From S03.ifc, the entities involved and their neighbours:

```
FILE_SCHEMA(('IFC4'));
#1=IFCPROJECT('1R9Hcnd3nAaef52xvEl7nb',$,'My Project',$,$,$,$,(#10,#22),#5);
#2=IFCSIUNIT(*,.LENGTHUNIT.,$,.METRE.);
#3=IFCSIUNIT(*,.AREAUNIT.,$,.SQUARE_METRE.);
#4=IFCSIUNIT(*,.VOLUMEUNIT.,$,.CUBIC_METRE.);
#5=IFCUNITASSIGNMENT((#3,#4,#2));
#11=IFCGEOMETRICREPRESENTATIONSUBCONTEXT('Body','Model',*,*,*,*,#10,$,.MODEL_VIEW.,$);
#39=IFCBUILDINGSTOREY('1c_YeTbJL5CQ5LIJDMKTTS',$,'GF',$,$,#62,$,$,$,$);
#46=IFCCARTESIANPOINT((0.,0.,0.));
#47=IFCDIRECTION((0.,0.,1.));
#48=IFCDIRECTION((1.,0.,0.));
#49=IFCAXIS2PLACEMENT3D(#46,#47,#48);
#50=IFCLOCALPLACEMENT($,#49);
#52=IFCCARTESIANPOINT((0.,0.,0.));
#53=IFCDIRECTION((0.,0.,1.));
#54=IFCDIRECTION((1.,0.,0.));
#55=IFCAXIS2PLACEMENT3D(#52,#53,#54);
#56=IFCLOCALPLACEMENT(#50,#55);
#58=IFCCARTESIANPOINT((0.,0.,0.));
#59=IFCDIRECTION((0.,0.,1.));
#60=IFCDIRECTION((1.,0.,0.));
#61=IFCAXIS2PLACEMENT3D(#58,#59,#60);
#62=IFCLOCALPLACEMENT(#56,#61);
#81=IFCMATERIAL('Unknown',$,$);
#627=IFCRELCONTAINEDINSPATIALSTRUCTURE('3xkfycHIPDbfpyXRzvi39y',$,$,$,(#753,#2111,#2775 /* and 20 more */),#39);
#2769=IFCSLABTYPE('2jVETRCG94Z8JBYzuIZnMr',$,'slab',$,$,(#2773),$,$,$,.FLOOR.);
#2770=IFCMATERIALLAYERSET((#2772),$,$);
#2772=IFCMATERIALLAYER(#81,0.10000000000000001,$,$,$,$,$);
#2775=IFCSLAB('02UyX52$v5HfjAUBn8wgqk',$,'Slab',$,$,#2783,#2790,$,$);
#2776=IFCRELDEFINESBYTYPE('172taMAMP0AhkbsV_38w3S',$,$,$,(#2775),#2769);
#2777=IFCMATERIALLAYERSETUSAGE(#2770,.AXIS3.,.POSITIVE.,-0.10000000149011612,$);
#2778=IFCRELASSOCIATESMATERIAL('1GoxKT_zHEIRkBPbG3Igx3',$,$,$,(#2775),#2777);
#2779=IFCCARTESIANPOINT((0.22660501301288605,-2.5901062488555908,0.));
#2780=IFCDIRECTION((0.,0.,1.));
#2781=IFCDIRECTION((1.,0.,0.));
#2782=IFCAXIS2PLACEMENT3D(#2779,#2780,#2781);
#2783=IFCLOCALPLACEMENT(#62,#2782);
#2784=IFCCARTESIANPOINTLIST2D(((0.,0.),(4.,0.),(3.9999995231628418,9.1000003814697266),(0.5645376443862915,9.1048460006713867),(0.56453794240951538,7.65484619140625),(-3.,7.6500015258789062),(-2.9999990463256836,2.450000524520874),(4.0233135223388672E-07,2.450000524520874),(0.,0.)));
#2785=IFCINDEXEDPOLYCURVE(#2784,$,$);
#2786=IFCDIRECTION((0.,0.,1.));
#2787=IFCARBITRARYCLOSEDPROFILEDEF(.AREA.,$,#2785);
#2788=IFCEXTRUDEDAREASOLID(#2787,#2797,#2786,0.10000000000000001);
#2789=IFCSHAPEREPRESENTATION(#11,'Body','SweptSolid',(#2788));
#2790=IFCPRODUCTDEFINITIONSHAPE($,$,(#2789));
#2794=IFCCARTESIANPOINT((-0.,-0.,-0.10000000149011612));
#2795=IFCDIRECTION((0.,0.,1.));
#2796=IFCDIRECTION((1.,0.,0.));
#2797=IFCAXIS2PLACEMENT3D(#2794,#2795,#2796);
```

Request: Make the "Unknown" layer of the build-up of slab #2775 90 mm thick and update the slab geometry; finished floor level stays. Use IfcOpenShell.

```python
import ifcopenshell
import ifcopenshell.util.element
import ifcopenshell.util.representation

model = ifcopenshell.open("S03.ifc")

layer_set = model.by_id(2770)
layer = next(l for l in layer_set.MaterialLayers if l.Material and l.Material.Name == "Unknown")
change = 0.09 - layer.LayerThickness
layer.LayerThickness += change

# Geometry does not follow the layer set by itself.
slabs = [e for e in ifcopenshell.util.element.get_elements_by_material(model, layer_set) if e.is_a("IfcSlab")]
for slab in sorted(slabs, key=lambda e: e.id()):
    body = ifcopenshell.util.representation.get_representation(slab, "Model", "Body")
    solid = body.Items[0]
    old_depth = solid.Depth
    solid.Depth += change
    # Extruded upwards: lower the start of the extrusion so the top stays.
    x, y, z = solid.Position.Location.Coordinates
    solid.Position.Location = model.createIfcCartesianPoint((x, y, z - change))
    print(slab.id(), f"{old_depth:g} -> {solid.Depth:g}")

# The layers are counted up from the underside, which has moved.
for usage in {ifcopenshell.util.element.get_material(slab) for slab in slabs}:
    usage.OffsetFromReferenceLine -= change

model.write("S03_rev.ifc")
```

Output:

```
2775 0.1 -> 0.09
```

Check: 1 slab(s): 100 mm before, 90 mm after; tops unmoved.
